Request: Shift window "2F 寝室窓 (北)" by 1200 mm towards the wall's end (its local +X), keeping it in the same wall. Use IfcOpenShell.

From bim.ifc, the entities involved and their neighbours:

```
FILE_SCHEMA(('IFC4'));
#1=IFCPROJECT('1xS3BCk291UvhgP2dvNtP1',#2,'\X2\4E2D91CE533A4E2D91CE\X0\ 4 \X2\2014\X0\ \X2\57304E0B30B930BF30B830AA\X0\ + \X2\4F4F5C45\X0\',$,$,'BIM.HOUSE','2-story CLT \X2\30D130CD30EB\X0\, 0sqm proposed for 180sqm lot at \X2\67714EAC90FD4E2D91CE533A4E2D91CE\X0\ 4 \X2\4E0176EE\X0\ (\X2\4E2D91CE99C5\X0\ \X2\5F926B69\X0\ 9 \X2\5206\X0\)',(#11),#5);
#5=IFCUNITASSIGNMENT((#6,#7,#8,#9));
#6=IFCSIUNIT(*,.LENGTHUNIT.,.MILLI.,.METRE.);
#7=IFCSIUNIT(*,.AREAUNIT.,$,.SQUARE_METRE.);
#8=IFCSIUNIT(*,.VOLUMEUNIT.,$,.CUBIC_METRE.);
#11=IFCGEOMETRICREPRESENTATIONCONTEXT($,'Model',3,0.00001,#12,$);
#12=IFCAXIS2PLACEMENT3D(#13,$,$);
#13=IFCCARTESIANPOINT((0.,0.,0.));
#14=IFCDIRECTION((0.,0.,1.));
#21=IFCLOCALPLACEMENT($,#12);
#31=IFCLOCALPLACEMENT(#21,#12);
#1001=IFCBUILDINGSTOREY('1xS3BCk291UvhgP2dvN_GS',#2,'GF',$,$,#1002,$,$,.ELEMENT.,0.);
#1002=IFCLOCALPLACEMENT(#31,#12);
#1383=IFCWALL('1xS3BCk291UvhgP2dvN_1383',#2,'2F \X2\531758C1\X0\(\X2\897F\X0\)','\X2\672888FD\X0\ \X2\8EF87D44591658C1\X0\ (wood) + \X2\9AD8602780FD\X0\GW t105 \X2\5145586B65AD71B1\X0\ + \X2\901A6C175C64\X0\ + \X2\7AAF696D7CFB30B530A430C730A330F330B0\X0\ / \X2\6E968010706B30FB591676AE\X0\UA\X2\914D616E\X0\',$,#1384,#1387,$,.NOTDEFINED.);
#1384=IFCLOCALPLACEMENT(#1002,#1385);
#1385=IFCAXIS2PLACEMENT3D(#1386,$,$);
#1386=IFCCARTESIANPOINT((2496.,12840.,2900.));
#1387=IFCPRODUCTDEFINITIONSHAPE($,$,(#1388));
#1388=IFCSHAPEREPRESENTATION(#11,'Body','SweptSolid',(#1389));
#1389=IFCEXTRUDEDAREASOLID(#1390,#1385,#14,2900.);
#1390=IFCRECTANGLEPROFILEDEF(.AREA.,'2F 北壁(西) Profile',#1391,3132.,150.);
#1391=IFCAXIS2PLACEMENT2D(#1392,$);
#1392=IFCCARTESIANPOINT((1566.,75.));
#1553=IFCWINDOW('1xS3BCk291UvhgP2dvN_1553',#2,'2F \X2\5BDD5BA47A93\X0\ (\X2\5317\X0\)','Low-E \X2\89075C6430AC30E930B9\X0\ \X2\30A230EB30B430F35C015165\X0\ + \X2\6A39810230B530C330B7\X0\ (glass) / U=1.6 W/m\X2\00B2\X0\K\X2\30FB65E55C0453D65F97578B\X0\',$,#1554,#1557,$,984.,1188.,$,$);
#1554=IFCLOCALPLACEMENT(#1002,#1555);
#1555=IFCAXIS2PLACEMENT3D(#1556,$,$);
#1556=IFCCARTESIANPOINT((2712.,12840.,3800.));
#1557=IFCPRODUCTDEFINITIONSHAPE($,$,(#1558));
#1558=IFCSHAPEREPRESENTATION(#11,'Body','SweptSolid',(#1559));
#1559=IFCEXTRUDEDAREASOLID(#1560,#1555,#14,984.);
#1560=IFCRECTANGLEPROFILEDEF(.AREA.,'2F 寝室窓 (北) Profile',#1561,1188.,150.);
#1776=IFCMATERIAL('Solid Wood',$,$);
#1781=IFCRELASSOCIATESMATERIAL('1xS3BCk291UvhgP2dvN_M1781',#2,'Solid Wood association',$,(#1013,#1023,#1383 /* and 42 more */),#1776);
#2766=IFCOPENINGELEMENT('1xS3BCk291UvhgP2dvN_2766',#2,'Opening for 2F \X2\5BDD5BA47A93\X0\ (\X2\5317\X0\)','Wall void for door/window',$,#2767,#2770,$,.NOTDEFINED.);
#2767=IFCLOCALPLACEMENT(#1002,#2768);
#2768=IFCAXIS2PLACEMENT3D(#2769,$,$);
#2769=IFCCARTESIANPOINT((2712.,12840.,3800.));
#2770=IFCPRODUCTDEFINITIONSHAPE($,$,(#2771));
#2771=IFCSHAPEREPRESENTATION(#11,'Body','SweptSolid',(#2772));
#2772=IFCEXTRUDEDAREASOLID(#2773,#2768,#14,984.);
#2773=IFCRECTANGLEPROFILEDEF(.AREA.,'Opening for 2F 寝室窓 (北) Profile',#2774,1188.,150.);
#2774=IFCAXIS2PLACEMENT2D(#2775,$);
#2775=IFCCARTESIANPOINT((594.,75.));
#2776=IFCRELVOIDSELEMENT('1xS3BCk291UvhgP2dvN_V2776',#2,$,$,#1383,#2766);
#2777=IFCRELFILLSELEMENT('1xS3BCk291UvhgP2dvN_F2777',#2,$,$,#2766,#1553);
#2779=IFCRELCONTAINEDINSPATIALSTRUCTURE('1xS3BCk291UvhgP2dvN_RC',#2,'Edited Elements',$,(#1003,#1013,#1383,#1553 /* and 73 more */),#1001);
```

```python
import ifcopenshell
import ifcopenshell.api.geometry
import ifcopenshell.util.placement
import ifcopenshell.util.unit

model = ifcopenshell.open("bim.ifc")
unit_scale = ifcopenshell.util.unit.calculate_unit_scale(model)

window = model.by_id(1553)
opening = window.FillsVoids[0].RelatingOpeningElement
wall = opening.VoidsElements[0].RelatingBuildingElement

wall_matrix = ifcopenshell.util.placement.get_local_placement(wall.ObjectPlacement)
shift = wall_matrix[:3, 0] * 1.2 / unit_scale
before = ifcopenshell.util.placement.get_local_placement(window.ObjectPlacement)[:3, 3].copy()

# The window is not placed relative to its opening, so move both.
for product in (opening, window):
    matrix = ifcopenshell.util.placement.get_local_placement(product.ObjectPlacement)
    matrix[:3, 3] += shift
    ifcopenshell.api.geometry.edit_object_placement(model, product=product, matrix=matrix, is_si=False)

after = ifcopenshell.util.placement.get_local_placement(window.ObjectPlacement)[:3, 3]
print("window moved by", (after - before).round(3) + 0.0)

model.write("bim_updated.ifc")
```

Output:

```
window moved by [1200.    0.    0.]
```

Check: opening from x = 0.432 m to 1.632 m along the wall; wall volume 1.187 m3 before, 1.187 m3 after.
